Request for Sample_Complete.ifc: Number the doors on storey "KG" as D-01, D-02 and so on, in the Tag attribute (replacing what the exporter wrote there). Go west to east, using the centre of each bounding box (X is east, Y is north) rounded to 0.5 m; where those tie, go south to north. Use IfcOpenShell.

First a look at what the model holds.

```python
import ifcopenshell
import ifcopenshell.util.element
import ifcopenshell.util.placement

model = ifcopenshell.open("Sample_Complete.ifc")
print(model.schema)
storey = next(s for s in model.by_type("IfcBuildingStorey") if s.Name == "KG")
doors = [e for e in ifcopenshell.util.element.get_decomposition(storey) if e.is_a("IfcDoor")]
for e in sorted(doors, key=lambda e: e.id()):
    origin = ifcopenshell.util.placement.get_local_placement(e.ObjectPlacement)[:3, 3]
    print(e.id(), e.Tag, e.Name, origin.round(2) + 0.0, sep=" | ")
```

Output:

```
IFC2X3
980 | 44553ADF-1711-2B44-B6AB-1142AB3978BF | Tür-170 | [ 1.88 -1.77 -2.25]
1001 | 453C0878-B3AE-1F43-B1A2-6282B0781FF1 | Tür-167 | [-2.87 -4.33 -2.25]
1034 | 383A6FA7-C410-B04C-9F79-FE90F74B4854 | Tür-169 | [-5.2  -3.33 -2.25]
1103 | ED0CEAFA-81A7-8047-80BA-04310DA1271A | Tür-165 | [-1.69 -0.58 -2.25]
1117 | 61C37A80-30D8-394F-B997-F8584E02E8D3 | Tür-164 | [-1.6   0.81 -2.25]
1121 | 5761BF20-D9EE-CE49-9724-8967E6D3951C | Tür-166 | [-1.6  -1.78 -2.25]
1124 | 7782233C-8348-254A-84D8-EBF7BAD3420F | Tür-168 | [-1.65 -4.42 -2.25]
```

```python
import ifcopenshell
import ifcopenshell.geom
import ifcopenshell.util.element
import ifcopenshell.util.shape

model = ifcopenshell.open("Sample_Complete.ifc")
settings = ifcopenshell.geom.settings()
settings.set("use-world-coords", True)


def centre(element):
    shape = ifcopenshell.geom.create_shape(settings, element)
    return ifcopenshell.util.shape.get_bbox_centroid(shape.geometry)


storey = next(s for s in model.by_type("IfcBuildingStorey") if s.Name == "KG")
doors = [e for e in ifcopenshell.util.element.get_decomposition(storey) if e.is_a("IfcDoor")]

# Insertion points can sit at a corner or the storey origin, so sort by the geometry (in metres).
centres = {e: centre(e) for e in doors}
doors.sort(key=lambda e: (round(centres[e][0] / 0.5), centres[e][1]))

for i, e in enumerate(doors, start=1):
    number = f"D-{i:02d}"
    e.Tag = number
    print(e.id(), number)

model.write("Sample_Complete-out.ifc")
```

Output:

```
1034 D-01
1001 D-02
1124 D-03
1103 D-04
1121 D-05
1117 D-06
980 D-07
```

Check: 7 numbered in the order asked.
